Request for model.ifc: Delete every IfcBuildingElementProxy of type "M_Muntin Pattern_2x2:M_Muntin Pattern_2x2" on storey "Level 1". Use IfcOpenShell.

First a look at what the model holds.

```python
import ifcopenshell
import ifcopenshell.util.element

model = ifcopenshell.open("model.ifc")
print(model.schema)
storey = next(s for s in model.by_type("IfcBuildingStorey") if s.Name == "Level 1")
proxies = [e for e in ifcopenshell.util.element.get_decomposition(storey) if e.is_a("IfcBuildingElementProxy")]
seen = {}
for e in proxies:
    element_type = ifcopenshell.util.element.get_type(e)
    name = element_type.Name if element_type not in (None, e) else None
    seen[name] = seen.get(name, 0) + 1
for name, count in sorted(seen.items(), key=str):
    print(count, "x", name)
```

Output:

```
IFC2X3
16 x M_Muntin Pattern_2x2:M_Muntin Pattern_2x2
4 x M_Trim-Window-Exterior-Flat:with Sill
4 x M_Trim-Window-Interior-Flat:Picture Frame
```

```python
import ifcopenshell
import ifcopenshell.api.root
import ifcopenshell.util.element

model = ifcopenshell.open("model.ifc")

storey = next(s for s in model.by_type("IfcBuildingStorey") if s.Name == "Level 1")
proxies = [e for e in ifcopenshell.util.element.get_decomposition(storey) if e.is_a("IfcBuildingElementProxy")]
targets = [e for e in proxies if (t := ifcopenshell.util.element.get_type(e)) not in (None, e) and t.Name == "M_Muntin Pattern_2x2:M_Muntin Pattern_2x2"]

for e in targets:
    ifcopenshell.api.root.remove_product(model, product=e)
print(len(targets), "removed")

model.write("model-out.ifc")
```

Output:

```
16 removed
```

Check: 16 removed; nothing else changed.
